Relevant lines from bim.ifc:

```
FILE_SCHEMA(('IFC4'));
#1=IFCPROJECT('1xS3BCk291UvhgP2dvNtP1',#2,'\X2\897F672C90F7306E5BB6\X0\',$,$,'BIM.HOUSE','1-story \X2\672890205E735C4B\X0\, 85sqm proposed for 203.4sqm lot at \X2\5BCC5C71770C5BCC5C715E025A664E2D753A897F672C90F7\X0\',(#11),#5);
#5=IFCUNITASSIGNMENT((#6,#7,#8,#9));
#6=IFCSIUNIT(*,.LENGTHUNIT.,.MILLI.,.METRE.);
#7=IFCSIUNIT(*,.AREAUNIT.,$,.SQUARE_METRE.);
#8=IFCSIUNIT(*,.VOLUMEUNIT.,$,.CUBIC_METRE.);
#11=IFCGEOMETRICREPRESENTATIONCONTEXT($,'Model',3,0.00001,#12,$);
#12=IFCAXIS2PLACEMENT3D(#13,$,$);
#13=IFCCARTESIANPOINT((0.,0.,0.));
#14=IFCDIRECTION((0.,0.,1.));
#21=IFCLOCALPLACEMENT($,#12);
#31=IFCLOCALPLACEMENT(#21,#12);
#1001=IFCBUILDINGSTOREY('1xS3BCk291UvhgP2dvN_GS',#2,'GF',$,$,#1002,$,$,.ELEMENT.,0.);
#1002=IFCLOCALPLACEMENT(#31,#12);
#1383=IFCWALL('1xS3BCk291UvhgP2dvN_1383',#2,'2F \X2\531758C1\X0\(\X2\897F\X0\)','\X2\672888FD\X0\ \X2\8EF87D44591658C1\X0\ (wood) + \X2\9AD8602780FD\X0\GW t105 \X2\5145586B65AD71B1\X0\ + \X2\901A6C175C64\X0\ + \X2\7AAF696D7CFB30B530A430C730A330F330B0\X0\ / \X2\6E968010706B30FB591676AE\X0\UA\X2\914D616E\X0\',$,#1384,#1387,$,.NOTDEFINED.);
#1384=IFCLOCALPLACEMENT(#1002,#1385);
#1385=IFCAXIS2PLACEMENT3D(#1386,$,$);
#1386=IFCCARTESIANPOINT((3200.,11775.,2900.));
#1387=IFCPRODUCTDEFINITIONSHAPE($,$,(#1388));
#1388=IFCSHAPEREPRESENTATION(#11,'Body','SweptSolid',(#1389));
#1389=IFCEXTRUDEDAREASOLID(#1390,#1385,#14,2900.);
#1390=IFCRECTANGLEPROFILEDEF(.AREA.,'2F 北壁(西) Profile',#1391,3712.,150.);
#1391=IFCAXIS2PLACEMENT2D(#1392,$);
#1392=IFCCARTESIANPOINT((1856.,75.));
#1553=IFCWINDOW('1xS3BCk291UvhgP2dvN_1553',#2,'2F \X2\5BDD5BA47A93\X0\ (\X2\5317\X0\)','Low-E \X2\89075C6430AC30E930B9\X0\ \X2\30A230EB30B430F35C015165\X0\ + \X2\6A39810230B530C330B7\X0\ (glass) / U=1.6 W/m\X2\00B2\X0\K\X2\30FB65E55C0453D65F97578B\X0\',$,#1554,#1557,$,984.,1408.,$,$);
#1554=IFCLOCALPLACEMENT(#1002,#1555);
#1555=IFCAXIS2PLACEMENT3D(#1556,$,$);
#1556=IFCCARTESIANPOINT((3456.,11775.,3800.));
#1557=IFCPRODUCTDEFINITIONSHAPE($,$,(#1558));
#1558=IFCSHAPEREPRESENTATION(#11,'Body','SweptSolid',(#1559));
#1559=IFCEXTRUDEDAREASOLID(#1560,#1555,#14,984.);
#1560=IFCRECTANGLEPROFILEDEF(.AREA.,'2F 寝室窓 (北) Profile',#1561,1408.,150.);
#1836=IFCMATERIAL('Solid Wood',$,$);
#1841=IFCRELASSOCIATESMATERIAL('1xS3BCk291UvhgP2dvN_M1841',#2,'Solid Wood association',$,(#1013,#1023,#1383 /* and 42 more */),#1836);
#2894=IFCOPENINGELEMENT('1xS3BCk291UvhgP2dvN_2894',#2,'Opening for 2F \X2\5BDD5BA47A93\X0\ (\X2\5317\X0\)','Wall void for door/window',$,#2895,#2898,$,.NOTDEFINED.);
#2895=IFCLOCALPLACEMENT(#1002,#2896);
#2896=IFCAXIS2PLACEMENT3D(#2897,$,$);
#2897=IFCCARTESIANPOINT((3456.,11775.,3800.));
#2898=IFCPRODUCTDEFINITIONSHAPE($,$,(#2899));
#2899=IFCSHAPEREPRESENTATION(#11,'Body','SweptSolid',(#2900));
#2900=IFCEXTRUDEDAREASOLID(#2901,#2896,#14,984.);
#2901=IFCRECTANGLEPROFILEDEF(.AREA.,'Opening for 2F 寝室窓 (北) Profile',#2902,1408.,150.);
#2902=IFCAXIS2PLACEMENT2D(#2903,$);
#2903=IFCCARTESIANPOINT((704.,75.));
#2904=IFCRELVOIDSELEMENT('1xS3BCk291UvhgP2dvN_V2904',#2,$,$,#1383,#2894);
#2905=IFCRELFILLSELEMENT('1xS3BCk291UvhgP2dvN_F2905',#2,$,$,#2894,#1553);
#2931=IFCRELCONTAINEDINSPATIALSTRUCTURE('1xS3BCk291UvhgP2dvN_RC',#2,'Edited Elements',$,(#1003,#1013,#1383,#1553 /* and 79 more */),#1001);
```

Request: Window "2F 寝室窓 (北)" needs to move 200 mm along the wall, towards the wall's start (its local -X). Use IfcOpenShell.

```python
import ifcopenshell
import ifcopenshell.api.geometry
import ifcopenshell.util.placement
import ifcopenshell.util.unit

model = ifcopenshell.open("bim.ifc")
unit_scale = ifcopenshell.util.unit.calculate_unit_scale(model)

window = model.by_guid("1xS3BCk291UvhgP2dvN_1553")
opening = window.FillsVoids[0].RelatingOpeningElement
wall = opening.VoidsElements[0].RelatingBuildingElement

wall_matrix = ifcopenshell.util.placement.get_local_placement(wall.ObjectPlacement)
shift = wall_matrix[:3, 0] * -0.2 / unit_scale
before = ifcopenshell.util.placement.get_local_placement(window.ObjectPlacement)[:3, 3].copy()

# The window is not placed relative to its opening, so move both.
for product in (opening, window):
    matrix = ifcopenshell.util.placement.get_local_placement(product.ObjectPlacement)
    matrix[:3, 3] += shift
    ifcopenshell.api.geometry.edit_object_placement(model, product=product, matrix=matrix, is_si=False)

after = ifcopenshell.util.placement.get_local_placement(window.ObjectPlacement)[:3, 3]
print("window moved by", (after - before).round(3) + 0.0)

model.write("bim_edited.ifc")
```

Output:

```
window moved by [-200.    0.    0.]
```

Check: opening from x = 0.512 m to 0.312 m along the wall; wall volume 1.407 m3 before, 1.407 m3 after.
